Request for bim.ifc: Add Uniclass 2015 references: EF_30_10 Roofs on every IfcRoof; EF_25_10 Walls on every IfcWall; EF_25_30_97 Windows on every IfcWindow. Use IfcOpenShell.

First a look at what the model holds.

```python
import ifcopenshell

model = ifcopenshell.open("bim.ifc")
print(model.schema)
print("classifications:", [c.Name for c in model.by_type("IfcClassification")])
for ifc_class in ("IfcDoor", "IfcRoof", "IfcStair", "IfcWall", "IfcWindow"):
    print(ifc_class, len(model.by_type(ifc_class)))
```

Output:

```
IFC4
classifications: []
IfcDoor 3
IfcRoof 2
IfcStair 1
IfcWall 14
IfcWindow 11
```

```python
import ifcopenshell
import ifcopenshell.api.classification

model = ifcopenshell.open("bim.ifc")

system = ifcopenshell.api.classification.add_classification(model, classification="Uniclass 2015")

codes = {
    "IfcRoof": ("EF_30_10", "Roofs"),
    "IfcWall": ("EF_25_10", "Walls"),
    "IfcWindow": ("EF_25_30_97", "Windows"),
}
for ifc_class, (code, name) in codes.items():
    products = model.by_type(ifc_class)
    ifcopenshell.api.classification.add_reference(
        model, products=products, classification=system, identification=code, name=name
    )
    print(code, len(products))

model.write("bim_v2.ifc")
```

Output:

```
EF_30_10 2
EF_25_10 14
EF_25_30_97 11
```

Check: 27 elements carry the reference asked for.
